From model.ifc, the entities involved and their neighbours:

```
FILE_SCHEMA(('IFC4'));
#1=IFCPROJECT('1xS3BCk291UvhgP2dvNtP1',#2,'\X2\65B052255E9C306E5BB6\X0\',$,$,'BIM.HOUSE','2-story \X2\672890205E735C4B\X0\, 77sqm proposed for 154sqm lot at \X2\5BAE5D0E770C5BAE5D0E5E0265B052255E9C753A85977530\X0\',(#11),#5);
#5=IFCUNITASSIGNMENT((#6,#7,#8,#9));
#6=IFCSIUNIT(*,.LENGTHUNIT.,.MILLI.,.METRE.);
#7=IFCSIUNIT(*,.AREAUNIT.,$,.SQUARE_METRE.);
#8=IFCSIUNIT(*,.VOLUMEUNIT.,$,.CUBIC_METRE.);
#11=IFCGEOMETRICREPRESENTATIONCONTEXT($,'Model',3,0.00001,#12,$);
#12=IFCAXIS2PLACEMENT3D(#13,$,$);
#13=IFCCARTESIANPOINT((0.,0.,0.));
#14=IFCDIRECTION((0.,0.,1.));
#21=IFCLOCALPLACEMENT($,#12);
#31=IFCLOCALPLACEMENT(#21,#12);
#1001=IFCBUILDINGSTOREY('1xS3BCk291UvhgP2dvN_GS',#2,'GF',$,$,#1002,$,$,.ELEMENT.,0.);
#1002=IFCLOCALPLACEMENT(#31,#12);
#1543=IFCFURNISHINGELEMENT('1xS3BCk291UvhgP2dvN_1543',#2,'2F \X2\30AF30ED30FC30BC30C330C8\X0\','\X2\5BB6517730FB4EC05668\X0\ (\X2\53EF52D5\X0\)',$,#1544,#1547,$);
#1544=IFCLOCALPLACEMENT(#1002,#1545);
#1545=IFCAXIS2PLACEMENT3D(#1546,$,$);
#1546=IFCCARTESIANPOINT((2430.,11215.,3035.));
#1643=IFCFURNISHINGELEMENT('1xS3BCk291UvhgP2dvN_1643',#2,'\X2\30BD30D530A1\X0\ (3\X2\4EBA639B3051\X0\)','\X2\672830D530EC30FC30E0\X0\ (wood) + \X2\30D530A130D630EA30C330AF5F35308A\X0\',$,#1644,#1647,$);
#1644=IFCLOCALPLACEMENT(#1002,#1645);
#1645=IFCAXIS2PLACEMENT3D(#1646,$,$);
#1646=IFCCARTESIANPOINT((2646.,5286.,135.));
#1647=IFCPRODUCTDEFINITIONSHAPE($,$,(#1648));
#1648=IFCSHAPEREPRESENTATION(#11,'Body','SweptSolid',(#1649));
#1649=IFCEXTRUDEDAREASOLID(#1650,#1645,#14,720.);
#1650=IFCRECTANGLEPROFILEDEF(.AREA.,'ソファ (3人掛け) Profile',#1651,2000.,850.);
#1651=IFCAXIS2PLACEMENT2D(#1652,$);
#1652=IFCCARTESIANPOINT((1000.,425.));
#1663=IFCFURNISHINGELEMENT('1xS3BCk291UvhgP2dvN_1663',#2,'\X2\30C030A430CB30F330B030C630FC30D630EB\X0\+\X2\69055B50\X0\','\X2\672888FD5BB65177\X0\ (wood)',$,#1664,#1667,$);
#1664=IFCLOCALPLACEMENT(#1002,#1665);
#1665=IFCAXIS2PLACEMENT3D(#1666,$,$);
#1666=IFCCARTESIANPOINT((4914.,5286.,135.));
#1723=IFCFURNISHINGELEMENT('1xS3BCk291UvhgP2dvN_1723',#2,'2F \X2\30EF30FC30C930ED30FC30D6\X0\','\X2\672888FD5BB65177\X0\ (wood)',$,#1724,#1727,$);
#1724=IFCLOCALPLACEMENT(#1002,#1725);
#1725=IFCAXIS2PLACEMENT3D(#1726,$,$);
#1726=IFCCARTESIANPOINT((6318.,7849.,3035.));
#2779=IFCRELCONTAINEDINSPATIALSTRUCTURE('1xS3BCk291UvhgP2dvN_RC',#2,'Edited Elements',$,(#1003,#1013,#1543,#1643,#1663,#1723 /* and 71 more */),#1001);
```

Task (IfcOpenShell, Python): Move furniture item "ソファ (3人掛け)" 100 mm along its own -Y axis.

```python
import ifcopenshell
import ifcopenshell.api.geometry
import ifcopenshell.util.placement

model = ifcopenshell.open("model.ifc")

item = model.by_id(1643)
matrix = ifcopenshell.util.placement.get_local_placement(item.ObjectPlacement)
matrix[:3, 3] -= matrix[:3, 1] * 100.0
ifcopenshell.api.geometry.edit_object_placement(model, product=item, matrix=matrix, is_si=False)

print(ifcopenshell.util.placement.get_local_placement(item.ObjectPlacement).round(3) + 0.0)

model.write("model_v2.ifc")
```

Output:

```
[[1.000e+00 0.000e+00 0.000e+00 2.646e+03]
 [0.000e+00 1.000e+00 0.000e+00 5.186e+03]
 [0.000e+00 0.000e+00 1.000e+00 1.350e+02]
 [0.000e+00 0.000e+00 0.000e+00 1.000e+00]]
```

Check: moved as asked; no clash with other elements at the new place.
